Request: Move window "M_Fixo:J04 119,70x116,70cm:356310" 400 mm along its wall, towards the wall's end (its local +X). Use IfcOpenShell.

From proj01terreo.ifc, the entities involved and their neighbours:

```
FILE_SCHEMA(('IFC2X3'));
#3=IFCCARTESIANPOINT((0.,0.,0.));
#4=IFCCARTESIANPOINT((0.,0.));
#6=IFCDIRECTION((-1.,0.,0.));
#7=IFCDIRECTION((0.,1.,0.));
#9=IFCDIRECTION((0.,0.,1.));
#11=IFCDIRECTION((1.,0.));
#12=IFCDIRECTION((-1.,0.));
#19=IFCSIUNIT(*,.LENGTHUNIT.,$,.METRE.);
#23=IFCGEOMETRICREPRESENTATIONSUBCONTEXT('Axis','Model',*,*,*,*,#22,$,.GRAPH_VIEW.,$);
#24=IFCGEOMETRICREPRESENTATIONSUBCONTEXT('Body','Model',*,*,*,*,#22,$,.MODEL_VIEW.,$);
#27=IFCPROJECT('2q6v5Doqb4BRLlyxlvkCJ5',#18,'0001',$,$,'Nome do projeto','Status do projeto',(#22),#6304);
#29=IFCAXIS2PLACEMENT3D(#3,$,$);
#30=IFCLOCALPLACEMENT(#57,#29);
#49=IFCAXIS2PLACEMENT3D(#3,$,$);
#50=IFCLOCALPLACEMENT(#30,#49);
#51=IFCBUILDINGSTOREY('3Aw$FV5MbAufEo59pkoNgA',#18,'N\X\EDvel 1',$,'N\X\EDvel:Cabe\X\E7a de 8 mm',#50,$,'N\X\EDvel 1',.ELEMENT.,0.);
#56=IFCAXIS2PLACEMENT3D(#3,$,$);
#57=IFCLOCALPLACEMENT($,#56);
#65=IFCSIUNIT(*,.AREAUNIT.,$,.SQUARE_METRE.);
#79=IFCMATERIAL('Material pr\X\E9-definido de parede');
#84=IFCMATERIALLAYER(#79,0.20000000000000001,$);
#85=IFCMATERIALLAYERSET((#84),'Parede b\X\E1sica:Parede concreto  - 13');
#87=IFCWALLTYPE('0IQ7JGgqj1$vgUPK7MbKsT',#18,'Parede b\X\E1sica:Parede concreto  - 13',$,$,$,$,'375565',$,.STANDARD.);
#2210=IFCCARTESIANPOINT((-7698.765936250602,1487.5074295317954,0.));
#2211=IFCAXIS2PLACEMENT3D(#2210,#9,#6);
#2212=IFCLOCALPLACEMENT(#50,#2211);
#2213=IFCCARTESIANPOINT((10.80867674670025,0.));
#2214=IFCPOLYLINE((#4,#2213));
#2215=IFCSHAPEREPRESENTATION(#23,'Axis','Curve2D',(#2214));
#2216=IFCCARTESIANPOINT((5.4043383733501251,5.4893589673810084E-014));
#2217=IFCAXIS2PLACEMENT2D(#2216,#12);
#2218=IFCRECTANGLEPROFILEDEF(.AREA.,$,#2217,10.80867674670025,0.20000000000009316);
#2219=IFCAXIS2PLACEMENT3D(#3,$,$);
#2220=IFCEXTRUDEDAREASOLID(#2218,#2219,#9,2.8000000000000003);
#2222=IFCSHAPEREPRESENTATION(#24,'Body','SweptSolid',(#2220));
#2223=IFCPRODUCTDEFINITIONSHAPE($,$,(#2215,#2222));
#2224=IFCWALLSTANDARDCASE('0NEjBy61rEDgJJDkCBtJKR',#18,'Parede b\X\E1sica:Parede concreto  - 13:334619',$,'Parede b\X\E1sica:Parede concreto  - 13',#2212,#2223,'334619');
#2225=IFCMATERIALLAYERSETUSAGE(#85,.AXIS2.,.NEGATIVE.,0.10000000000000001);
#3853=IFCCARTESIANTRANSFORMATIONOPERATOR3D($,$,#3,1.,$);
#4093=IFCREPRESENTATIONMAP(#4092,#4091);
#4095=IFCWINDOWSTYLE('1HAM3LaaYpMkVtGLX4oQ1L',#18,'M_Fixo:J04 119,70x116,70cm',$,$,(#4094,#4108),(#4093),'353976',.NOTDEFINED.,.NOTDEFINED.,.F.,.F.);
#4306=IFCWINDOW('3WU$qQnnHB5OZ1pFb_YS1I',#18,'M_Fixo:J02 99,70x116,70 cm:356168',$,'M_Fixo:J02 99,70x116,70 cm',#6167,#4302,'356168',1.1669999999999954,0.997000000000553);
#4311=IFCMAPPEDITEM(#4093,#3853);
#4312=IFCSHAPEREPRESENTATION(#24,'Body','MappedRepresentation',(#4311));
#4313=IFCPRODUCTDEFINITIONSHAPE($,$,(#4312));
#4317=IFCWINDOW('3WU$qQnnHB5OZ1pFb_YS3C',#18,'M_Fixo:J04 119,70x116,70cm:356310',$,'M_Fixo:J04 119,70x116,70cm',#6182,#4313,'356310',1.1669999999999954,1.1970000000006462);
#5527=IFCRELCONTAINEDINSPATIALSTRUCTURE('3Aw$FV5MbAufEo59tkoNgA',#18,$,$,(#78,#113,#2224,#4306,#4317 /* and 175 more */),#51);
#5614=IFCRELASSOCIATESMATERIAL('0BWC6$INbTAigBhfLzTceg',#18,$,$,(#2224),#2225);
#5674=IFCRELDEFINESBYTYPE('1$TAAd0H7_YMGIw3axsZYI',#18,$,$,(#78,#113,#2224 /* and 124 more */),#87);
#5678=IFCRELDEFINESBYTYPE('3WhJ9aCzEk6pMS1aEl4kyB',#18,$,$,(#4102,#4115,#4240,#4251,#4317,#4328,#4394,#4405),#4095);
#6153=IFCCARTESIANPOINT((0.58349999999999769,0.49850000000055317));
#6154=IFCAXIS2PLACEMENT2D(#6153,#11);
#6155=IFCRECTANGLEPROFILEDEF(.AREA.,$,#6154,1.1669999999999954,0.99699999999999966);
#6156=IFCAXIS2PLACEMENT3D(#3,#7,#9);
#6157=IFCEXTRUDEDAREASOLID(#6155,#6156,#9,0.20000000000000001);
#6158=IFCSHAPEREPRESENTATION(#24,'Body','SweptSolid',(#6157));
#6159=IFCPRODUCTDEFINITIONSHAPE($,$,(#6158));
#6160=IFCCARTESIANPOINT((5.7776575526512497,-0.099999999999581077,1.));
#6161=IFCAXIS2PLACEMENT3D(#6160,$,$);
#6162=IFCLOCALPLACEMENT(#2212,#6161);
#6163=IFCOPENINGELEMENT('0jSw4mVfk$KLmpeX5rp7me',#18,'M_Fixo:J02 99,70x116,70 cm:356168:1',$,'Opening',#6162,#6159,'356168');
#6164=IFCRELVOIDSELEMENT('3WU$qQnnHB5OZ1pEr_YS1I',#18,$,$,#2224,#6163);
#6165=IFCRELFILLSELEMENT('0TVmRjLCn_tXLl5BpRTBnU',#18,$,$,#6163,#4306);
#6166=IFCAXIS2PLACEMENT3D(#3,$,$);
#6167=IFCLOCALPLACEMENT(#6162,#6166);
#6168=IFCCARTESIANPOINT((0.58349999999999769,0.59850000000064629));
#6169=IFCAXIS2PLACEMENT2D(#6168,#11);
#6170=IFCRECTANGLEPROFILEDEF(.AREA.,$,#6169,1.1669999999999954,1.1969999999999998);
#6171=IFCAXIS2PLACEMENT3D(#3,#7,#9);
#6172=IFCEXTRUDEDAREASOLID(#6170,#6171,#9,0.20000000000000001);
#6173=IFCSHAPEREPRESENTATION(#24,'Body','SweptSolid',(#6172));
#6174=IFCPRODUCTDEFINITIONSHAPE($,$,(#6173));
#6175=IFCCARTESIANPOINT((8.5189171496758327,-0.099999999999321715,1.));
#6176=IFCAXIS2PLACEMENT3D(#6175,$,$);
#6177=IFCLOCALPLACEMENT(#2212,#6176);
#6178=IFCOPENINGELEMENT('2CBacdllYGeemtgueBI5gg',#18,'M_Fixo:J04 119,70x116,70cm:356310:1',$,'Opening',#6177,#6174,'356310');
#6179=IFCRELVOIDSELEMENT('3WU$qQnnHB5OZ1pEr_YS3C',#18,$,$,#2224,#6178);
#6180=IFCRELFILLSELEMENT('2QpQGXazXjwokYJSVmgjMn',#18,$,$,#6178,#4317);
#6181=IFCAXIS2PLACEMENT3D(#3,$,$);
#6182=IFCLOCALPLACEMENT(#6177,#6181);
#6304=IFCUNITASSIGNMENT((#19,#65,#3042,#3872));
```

```python
import ifcopenshell
import ifcopenshell.api.geometry
import ifcopenshell.util.placement

model = ifcopenshell.open("proj01terreo.ifc")

window = model.by_guid("3WU$qQnnHB5OZ1pFb_YS3C")
opening = window.FillsVoids[0].RelatingOpeningElement
wall = opening.VoidsElements[0].RelatingBuildingElement

wall_matrix = ifcopenshell.util.placement.get_local_placement(wall.ObjectPlacement)
shift = wall_matrix[:3, 0] * 0.4
before = ifcopenshell.util.placement.get_local_placement(window.ObjectPlacement)[:3, 3].copy()

# The window is placed relative to its opening, so it follows when the opening moves.
matrix = ifcopenshell.util.placement.get_local_placement(opening.ObjectPlacement)
matrix[:3, 3] += shift
ifcopenshell.api.geometry.edit_object_placement(
    model, product=opening, matrix=matrix, is_si=False, should_transform_children=True
)

after = ifcopenshell.util.placement.get_local_placement(window.ObjectPlacement)[:3, 3]
print("window moved by", (after - before).round(3) + 0.0)

model.write("proj01terreo_v2.ifc")
```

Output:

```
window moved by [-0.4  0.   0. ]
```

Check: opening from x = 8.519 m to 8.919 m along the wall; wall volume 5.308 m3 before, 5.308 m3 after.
